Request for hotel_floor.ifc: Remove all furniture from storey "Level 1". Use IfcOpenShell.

First a look at what the model holds.

```python
import ifcopenshell
import ifcopenshell.util.element

model = ifcopenshell.open("hotel_floor.ifc")
print(model.schema)
storey = next(s for s in model.by_type("IfcBuildingStorey") if s.Name == "Level 1")
furniture = [e for e in ifcopenshell.util.element.get_decomposition(storey) if e.is_a("IfcFurnishingElement")]
seen = {}
for e in furniture:
    element_type = ifcopenshell.util.element.get_type(e)
    name = element_type.Name if element_type not in (None, e) else None
    seen[name] = seen.get(name, 0) + 1
for name, count in sorted(seen.items(), key=str):
    print(count, "x", name)
```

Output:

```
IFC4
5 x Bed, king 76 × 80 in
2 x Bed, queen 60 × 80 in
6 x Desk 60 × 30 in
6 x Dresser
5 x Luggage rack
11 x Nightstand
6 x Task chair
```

```python
import ifcopenshell
import ifcopenshell.api.root
import ifcopenshell.util.element

model = ifcopenshell.open("hotel_floor.ifc")

storey = next(s for s in model.by_type("IfcBuildingStorey") if s.Name == "Level 1")
furniture = [e for e in ifcopenshell.util.element.get_decomposition(storey) if e.is_a("IfcFurnishingElement")]

for e in furniture:
    ifcopenshell.api.root.remove_product(model, product=e)
print(len(furniture), "removed")

model.write("hotel_floor_rev.ifc")
```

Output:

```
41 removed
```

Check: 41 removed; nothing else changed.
